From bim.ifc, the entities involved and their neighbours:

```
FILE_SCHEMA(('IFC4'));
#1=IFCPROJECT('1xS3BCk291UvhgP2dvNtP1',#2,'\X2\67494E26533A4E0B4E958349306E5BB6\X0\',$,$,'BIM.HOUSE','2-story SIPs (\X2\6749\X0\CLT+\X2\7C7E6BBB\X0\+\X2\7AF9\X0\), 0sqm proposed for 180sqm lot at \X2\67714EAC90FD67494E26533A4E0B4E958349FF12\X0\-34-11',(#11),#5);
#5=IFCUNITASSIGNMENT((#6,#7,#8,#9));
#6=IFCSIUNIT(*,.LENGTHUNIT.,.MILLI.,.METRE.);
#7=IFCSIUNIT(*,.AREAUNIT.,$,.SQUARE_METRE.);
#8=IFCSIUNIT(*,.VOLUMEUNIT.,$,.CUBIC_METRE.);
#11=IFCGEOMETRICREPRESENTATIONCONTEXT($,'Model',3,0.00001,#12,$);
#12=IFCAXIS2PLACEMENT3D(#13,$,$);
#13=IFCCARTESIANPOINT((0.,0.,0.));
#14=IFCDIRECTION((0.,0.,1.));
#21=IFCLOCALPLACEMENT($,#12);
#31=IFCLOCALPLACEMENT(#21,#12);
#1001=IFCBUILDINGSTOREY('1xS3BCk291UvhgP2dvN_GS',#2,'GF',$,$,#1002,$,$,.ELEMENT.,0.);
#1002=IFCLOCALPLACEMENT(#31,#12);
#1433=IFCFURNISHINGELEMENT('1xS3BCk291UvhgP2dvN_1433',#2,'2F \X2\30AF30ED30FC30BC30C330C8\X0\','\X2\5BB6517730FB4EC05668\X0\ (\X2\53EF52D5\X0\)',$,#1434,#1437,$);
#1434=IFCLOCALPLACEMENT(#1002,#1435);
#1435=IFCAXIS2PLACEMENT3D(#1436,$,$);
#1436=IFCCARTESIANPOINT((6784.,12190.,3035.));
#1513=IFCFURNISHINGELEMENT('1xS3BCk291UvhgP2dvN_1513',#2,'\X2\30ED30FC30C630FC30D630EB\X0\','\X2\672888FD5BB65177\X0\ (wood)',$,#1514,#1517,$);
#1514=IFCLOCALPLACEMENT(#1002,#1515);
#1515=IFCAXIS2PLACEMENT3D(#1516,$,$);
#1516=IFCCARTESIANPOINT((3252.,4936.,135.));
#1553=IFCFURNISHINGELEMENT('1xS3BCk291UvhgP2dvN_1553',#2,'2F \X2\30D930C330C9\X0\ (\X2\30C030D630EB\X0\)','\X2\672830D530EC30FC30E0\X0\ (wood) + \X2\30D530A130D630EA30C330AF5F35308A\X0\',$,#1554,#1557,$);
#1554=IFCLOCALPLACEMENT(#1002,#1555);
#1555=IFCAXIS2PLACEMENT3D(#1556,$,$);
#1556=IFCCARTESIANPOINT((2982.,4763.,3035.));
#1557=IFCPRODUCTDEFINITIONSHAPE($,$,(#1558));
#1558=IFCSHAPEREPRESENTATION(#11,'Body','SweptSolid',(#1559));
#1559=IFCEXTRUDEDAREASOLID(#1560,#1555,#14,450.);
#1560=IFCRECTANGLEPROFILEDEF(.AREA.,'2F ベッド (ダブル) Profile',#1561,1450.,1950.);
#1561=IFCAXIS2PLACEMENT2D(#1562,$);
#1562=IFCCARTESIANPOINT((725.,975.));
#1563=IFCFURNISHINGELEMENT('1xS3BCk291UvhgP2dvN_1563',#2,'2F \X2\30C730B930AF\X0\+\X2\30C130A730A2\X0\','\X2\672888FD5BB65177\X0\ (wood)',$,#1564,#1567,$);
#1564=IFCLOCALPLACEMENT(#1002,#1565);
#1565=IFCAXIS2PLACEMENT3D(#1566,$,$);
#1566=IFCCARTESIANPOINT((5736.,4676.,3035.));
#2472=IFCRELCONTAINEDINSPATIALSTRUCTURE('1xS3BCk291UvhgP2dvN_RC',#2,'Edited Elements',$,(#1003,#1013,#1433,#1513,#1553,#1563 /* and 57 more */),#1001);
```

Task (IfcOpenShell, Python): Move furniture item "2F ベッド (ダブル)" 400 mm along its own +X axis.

```python
import ifcopenshell
import ifcopenshell.api.geometry
import ifcopenshell.util.placement

model = ifcopenshell.open("bim.ifc")

item = model.by_id(1553)
matrix = ifcopenshell.util.placement.get_local_placement(item.ObjectPlacement)
matrix[:3, 3] += matrix[:3, 0] * 400.0
ifcopenshell.api.geometry.edit_object_placement(model, product=item, matrix=matrix, is_si=False)

print(ifcopenshell.util.placement.get_local_placement(item.ObjectPlacement).round(3) + 0.0)

model.write("bim_v2.ifc")
```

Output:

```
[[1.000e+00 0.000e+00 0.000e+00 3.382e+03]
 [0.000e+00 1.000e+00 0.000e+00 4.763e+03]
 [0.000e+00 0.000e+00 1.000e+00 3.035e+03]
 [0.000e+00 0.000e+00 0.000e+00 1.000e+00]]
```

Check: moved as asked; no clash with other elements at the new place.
